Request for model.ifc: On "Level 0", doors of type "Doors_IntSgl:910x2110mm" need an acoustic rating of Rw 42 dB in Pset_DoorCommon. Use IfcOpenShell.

First a look at what the model holds.

```python
import ifcopenshell
import ifcopenshell.util.element

model = ifcopenshell.open("model.ifc")
print(model.schema)
storey = next(s for s in model.by_type("IfcBuildingStorey") if s.Name == "Level 0")
doors = [e for e in ifcopenshell.util.element.get_decomposition(storey) if e.is_a("IfcDoor")]
seen = {}
for e in doors:
    element_type = ifcopenshell.util.element.get_type(e)
    key = (element_type.Name if element_type != e and element_type else None, ifcopenshell.util.element.get_pset(e, "Pset_DoorCommon", "AcousticRating"))
    seen[key] = seen.get(key, 0) + 1
for (name, value), count in sorted(seen.items(), key=str):
    print(count, "x", name, "|", value)
```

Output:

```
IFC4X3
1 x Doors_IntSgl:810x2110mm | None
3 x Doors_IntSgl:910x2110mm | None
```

```python
import ifcopenshell
import ifcopenshell.api.pset
import ifcopenshell.util.element

model = ifcopenshell.open("model.ifc")

storey = next(s for s in model.by_type("IfcBuildingStorey") if s.Name == "Level 0")
doors = [e for e in ifcopenshell.util.element.get_decomposition(storey) if e.is_a("IfcDoor")]

count = 0
for e in doors:
    element_type = ifcopenshell.util.element.get_type(e)
    if element_type in (None, e) or element_type.Name != "Doors_IntSgl:910x2110mm":
        continue
    # add_pset returns the element's existing set when there is one.
    pset = ifcopenshell.api.pset.add_pset(model, product=e, name="Pset_DoorCommon")
    ifcopenshell.api.pset.edit_pset(model, pset=pset, properties={"AcousticRating": "Rw 42 dB"})
    count += 1

print(count, "doors updated")

model.write("model_v2.ifc")
```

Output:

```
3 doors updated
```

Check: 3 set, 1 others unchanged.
